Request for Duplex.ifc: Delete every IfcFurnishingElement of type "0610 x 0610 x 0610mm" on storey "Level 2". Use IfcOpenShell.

First a look at what the model holds.

```python
import ifcopenshell
import ifcopenshell.util.element

model = ifcopenshell.open("Duplex.ifc")
print(model.schema)
storey = next(s for s in model.by_type("IfcBuildingStorey") if s.Name == "Level 2")
furniture = [e for e in ifcopenshell.util.element.get_decomposition(storey) if e.is_a("IfcFurnishingElement")]
seen = {}
for e in furniture:
    element_type = ifcopenshell.util.element.get_type(e)
    name = element_type.Name if element_type not in (None, e) else None
    seen[name] = seen.get(name, 0) + 1
for name, count in sorted(seen.items(), key=str):
    print(count, "x", name)
```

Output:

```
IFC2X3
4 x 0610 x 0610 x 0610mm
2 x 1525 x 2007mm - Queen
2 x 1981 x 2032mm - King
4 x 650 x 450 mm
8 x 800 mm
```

```python
import ifcopenshell
import ifcopenshell.api.root
import ifcopenshell.util.element

model = ifcopenshell.open("Duplex.ifc")

storey = next(s for s in model.by_type("IfcBuildingStorey") if s.Name == "Level 2")
furniture = [e for e in ifcopenshell.util.element.get_decomposition(storey) if e.is_a("IfcFurnishingElement")]
targets = [e for e in furniture if (t := ifcopenshell.util.element.get_type(e)) not in (None, e) and t.Name == "0610 x 0610 x 0610mm"]

for e in targets:
    ifcopenshell.api.root.remove_product(model, product=e)
print(len(targets), "removed")

model.write("Duplex_v2.ifc")
```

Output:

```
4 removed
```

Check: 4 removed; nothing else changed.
